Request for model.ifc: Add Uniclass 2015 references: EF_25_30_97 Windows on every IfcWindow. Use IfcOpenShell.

First a look at what the model holds.

```python
import ifcopenshell

model = ifcopenshell.open("model.ifc")
print(model.schema)
print("classifications:", [c.Name for c in model.by_type("IfcClassification")])
for ifc_class in ("IfcDoor", "IfcRoof", "IfcStair", "IfcWall", "IfcWindow"):
    print(ifc_class, len(model.by_type(ifc_class)))
```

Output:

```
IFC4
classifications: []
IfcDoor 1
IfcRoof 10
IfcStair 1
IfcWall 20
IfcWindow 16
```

```python
import ifcopenshell
import ifcopenshell.api.classification

model = ifcopenshell.open("model.ifc")

system = ifcopenshell.api.classification.add_classification(model, classification="Uniclass 2015")

codes = {
    "IfcWindow": ("EF_25_30_97", "Windows"),
}
for ifc_class, (code, name) in codes.items():
    products = model.by_type(ifc_class)
    ifcopenshell.api.classification.add_reference(
        model, products=products, classification=system, identification=code, name=name
    )
    print(code, len(products))

model.write("model_v2.ifc")
```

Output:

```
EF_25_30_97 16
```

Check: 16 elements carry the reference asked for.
